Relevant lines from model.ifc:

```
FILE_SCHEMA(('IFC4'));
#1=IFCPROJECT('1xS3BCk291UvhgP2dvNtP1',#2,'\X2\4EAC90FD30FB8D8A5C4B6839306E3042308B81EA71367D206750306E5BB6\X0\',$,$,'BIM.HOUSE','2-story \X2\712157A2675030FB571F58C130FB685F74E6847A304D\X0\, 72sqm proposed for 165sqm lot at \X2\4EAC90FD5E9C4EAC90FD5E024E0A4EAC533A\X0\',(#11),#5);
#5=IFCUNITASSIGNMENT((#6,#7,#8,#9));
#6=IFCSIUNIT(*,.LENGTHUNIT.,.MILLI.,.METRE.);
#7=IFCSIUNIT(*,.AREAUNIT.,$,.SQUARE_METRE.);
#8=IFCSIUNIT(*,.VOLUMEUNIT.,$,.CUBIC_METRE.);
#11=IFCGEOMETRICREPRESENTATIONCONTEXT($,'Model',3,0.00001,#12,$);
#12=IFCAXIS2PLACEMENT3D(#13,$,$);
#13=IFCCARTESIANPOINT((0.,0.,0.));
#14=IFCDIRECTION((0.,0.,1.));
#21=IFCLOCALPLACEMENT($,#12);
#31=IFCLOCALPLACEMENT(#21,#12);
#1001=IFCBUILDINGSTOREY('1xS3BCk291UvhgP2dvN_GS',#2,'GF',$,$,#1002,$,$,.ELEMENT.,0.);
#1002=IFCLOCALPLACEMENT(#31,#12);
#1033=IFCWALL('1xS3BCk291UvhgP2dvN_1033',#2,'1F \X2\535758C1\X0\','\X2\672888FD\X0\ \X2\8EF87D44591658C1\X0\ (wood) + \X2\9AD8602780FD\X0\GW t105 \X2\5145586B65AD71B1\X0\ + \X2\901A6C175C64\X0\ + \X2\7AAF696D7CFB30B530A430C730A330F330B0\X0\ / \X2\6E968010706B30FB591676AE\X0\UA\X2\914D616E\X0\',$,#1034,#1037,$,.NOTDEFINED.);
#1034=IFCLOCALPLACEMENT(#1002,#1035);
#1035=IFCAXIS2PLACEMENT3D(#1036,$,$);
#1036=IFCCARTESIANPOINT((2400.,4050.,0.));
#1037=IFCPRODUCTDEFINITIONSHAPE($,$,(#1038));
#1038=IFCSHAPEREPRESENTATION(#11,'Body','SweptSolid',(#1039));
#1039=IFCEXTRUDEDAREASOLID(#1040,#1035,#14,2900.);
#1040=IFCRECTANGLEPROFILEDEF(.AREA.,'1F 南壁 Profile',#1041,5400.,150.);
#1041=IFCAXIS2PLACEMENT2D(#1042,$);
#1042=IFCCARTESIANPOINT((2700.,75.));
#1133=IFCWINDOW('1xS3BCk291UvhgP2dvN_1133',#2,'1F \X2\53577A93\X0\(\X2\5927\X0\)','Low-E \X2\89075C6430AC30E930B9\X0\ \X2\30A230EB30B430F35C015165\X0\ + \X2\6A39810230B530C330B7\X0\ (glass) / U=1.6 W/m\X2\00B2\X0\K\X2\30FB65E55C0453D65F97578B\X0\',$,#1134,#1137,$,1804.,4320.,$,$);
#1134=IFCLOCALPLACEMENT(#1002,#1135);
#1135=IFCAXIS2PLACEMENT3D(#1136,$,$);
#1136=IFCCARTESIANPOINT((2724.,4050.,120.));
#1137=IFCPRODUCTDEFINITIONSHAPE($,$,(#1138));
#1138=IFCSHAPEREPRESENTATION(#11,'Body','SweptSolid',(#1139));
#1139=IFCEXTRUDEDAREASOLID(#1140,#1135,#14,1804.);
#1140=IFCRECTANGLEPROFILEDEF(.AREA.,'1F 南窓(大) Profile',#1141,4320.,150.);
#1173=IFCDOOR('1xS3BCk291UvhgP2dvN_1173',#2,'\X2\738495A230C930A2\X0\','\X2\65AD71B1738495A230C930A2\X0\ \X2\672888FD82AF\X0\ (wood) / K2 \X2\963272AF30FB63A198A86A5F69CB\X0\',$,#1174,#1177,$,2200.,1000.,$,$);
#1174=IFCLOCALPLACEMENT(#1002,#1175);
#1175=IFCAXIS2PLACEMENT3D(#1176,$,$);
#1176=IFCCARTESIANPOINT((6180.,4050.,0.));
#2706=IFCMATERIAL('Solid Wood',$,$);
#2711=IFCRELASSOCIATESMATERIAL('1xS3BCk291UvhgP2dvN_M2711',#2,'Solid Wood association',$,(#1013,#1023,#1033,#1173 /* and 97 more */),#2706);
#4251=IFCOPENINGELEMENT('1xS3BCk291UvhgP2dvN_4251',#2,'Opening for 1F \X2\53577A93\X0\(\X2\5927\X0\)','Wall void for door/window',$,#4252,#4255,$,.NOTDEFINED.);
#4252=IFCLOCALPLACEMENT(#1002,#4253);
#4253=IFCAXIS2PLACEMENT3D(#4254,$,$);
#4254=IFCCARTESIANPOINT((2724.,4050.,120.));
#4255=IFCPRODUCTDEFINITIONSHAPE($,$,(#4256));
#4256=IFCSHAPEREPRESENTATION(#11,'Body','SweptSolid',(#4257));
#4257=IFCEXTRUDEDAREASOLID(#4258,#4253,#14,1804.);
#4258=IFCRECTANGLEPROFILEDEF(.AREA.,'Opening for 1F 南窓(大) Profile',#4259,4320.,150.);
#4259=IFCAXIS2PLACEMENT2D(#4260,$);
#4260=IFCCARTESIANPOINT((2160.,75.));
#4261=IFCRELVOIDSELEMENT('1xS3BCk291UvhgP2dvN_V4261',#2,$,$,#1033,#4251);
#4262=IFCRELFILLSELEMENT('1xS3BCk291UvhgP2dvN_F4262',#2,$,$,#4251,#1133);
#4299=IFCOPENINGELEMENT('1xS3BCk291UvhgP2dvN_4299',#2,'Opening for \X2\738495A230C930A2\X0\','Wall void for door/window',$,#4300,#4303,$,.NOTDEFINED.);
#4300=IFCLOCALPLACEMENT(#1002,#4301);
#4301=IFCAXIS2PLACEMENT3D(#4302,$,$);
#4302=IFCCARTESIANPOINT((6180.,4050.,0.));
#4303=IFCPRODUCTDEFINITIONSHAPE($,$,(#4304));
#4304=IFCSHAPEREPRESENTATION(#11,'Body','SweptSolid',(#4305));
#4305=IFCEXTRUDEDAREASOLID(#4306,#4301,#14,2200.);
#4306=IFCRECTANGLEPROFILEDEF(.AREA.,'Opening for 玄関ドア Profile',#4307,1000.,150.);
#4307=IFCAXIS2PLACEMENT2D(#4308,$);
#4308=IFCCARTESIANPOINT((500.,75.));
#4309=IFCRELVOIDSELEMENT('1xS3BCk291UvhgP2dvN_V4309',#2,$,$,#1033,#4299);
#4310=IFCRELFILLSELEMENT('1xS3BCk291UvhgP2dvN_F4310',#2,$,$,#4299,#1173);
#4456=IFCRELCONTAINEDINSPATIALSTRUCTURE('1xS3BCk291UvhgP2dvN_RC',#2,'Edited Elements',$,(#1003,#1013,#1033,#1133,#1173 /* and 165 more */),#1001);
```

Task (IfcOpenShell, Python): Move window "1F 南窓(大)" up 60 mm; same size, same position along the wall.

```python
import numpy as np
import ifcopenshell
import ifcopenshell.api.geometry
import ifcopenshell.util.placement
import ifcopenshell.util.unit

model = ifcopenshell.open("model.ifc")
unit_scale = ifcopenshell.util.unit.calculate_unit_scale(model)

window = model.by_guid("1xS3BCk291UvhgP2dvN_1133")
opening = window.FillsVoids[0].RelatingOpeningElement
dz = 60.0

shift = np.array([0.0, 0.0, dz])
# The window is not placed relative to its opening, so move both.
for product in (opening, window):
    matrix = ifcopenshell.util.placement.get_local_placement(product.ObjectPlacement)
    matrix[:3, 3] += shift
    ifcopenshell.api.geometry.edit_object_placement(model, product=product, matrix=matrix, is_si=False)

print(f"moved by {dz * unit_scale:+.3f} m")

model.write("model_v2.ifc")
```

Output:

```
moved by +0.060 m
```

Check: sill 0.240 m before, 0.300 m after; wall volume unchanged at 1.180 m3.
